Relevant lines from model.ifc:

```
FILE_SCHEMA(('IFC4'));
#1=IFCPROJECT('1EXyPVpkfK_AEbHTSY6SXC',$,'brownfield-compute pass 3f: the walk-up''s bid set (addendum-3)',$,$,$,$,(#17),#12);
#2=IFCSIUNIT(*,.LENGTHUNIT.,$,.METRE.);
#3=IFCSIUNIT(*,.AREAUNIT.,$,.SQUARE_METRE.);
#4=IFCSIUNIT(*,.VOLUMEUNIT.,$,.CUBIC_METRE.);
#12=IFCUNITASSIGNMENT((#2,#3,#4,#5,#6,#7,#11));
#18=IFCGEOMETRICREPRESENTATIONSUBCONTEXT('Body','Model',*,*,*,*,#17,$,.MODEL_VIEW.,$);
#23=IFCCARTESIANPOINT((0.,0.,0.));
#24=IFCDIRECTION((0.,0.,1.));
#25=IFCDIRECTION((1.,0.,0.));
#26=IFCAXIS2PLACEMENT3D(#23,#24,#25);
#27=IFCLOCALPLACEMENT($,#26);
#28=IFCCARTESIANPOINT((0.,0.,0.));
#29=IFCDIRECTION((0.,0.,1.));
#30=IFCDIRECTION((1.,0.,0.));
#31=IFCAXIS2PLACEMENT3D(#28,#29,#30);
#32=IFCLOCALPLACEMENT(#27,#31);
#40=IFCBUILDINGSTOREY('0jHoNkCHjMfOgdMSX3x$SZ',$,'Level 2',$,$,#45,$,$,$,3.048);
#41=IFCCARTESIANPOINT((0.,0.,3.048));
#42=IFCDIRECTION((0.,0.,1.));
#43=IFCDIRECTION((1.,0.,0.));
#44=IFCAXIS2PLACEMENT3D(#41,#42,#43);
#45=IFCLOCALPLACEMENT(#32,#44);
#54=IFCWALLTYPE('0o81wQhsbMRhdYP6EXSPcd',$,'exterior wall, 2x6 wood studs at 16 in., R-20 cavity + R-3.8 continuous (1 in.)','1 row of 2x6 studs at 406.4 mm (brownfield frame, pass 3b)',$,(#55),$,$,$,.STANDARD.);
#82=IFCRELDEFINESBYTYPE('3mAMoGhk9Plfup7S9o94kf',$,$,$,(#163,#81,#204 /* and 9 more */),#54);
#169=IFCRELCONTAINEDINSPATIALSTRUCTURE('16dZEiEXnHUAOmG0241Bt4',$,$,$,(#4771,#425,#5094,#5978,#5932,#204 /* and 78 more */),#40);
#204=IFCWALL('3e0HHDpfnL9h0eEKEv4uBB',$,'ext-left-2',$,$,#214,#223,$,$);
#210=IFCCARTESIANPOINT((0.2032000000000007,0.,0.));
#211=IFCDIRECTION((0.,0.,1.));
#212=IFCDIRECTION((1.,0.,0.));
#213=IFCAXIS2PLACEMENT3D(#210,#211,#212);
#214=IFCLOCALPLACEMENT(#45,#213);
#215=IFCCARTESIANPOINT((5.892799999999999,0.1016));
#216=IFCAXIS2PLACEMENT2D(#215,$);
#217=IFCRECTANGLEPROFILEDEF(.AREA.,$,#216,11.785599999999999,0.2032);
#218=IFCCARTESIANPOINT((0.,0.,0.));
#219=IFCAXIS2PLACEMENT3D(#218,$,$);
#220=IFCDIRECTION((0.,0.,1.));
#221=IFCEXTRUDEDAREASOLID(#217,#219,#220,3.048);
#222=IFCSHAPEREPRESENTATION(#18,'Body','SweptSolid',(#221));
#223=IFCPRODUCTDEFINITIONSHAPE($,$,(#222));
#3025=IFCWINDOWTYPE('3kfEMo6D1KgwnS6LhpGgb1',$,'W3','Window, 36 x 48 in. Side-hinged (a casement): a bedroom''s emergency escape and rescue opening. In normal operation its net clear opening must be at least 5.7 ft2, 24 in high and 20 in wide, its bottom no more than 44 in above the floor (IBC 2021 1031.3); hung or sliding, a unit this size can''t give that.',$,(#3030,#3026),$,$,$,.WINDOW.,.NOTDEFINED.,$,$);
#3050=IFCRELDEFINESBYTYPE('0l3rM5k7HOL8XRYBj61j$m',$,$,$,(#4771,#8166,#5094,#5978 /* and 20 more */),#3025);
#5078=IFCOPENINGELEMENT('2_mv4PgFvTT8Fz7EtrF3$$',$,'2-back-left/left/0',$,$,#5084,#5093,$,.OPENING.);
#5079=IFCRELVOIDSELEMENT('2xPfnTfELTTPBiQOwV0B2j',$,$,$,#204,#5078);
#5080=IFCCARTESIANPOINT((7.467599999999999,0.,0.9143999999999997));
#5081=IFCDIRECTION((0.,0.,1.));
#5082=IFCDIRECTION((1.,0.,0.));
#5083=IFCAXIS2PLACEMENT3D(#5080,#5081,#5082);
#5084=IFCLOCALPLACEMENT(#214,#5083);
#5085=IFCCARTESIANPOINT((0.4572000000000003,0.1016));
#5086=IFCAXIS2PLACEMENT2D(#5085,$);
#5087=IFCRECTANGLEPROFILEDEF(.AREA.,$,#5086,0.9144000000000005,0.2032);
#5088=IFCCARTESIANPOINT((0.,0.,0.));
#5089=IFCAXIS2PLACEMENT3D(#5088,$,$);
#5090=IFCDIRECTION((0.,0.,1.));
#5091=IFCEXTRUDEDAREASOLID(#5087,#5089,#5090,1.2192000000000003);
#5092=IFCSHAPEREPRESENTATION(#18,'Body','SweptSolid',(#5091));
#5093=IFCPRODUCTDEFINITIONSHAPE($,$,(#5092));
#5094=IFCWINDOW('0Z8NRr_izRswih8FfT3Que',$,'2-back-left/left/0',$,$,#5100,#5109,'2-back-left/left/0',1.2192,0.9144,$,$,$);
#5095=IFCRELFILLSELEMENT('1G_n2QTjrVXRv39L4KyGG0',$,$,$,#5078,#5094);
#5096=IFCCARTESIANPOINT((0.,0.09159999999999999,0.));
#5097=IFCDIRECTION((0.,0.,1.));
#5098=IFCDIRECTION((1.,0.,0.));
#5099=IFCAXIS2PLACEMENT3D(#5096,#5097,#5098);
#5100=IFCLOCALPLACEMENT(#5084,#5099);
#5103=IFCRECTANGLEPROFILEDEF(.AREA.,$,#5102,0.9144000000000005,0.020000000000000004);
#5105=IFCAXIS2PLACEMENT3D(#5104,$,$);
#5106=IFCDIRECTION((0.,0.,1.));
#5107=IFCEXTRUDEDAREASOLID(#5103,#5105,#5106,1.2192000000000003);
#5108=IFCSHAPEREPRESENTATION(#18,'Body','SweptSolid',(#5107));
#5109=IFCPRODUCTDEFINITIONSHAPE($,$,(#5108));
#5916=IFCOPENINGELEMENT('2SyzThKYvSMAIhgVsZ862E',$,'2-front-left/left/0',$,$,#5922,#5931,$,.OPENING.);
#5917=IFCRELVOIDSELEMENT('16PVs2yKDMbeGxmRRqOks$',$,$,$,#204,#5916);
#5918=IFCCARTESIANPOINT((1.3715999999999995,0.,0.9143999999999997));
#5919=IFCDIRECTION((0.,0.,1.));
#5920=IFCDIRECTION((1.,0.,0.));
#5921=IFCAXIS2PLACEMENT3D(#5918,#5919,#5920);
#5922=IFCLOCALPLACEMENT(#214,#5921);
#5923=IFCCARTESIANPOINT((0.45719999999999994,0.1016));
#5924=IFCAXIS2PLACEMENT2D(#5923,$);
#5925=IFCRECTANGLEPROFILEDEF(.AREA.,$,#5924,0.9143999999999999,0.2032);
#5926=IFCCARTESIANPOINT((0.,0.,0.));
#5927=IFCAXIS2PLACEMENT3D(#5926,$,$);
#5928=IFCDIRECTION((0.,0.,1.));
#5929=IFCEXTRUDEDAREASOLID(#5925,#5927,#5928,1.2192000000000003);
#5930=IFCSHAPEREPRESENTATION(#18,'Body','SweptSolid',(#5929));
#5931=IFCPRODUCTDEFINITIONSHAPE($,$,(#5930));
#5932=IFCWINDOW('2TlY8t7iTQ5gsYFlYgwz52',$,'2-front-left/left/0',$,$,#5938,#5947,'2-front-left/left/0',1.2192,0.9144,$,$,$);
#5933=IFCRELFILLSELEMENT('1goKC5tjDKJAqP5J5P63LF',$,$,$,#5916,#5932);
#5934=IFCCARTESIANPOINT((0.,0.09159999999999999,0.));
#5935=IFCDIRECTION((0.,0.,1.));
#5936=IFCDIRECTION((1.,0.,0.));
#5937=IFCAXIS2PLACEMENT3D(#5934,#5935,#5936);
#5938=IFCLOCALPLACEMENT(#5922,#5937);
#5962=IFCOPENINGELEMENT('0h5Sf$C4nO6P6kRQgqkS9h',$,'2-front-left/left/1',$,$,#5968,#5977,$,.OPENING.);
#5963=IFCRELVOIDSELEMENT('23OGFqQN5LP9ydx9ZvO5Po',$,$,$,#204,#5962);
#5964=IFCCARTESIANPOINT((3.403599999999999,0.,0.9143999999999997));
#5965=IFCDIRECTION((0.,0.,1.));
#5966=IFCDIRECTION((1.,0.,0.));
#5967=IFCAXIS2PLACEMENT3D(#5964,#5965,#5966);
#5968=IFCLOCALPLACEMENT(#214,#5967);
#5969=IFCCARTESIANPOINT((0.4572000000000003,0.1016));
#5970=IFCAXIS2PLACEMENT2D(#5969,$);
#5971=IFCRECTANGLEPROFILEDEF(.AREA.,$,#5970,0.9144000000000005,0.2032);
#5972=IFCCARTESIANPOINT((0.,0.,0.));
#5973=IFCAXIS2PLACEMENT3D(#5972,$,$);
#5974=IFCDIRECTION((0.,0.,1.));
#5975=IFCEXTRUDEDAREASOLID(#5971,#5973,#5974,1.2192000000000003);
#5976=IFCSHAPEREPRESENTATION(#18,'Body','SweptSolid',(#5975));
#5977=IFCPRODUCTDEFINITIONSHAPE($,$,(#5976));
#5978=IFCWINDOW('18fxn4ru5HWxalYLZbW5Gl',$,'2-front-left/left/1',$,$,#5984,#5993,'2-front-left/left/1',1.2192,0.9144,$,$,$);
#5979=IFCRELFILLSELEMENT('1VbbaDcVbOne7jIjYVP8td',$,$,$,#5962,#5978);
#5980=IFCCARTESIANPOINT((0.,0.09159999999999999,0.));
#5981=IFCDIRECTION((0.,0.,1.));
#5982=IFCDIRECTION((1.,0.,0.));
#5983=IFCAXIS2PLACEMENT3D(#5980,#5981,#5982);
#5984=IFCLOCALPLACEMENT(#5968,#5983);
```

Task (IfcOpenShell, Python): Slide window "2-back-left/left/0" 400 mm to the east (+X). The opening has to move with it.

```python
import ifcopenshell
import ifcopenshell.api.geometry
import ifcopenshell.util.placement

model = ifcopenshell.open("model.ifc")

window = model.by_guid("0Z8NRr_izRswih8FfT3Que")
opening = window.FillsVoids[0].RelatingOpeningElement
wall = opening.VoidsElements[0].RelatingBuildingElement

wall_matrix = ifcopenshell.util.placement.get_local_placement(wall.ObjectPlacement)
shift = wall_matrix[:3, 0] * 0.4
before = ifcopenshell.util.placement.get_local_placement(window.ObjectPlacement)[:3, 3].copy()

# The window is placed relative to its opening, so it follows when the opening moves.
matrix = ifcopenshell.util.placement.get_local_placement(opening.ObjectPlacement)
matrix[:3, 3] += shift
ifcopenshell.api.geometry.edit_object_placement(
    model, product=opening, matrix=matrix, is_si=False, should_transform_children=True
)

after = ifcopenshell.util.placement.get_local_placement(window.ObjectPlacement)[:3, 3]
print("window moved by", (after - before).round(3) + 0.0)

model.write("model_updated.ifc")
```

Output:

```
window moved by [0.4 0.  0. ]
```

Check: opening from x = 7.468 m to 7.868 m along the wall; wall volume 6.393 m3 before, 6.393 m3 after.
